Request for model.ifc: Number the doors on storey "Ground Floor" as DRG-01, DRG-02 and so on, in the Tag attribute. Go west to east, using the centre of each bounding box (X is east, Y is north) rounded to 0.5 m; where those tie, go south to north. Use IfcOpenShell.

First a look at what the model holds.

```python
import ifcopenshell
import ifcopenshell.util.element
import ifcopenshell.util.placement

model = ifcopenshell.open("model.ifc")
print(model.schema)
storey = next(s for s in model.by_type("IfcBuildingStorey") if s.Name == "Ground Floor")
doors = [e for e in ifcopenshell.util.element.get_decomposition(storey) if e.is_a("IfcDoor")]
for e in sorted(doors, key=lambda e: e.id()):
    origin = ifcopenshell.util.placement.get_local_placement(e.ObjectPlacement)[:3, 3]
    print(e.id(), e.Tag, e.Name, origin.round(2) + 0.0, sep=" | ")
```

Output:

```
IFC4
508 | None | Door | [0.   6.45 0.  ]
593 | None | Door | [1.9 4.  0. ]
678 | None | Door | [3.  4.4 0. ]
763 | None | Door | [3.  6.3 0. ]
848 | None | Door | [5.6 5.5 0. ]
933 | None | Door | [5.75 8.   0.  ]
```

```python
import ifcopenshell
import ifcopenshell.geom
import ifcopenshell.util.element
import ifcopenshell.util.shape

model = ifcopenshell.open("model.ifc")
settings = ifcopenshell.geom.settings()
settings.set("use-world-coords", True)


def centre(element):
    shape = ifcopenshell.geom.create_shape(settings, element)
    return ifcopenshell.util.shape.get_bbox_centroid(shape.geometry)


storey = next(s for s in model.by_type("IfcBuildingStorey") if s.Name == "Ground Floor")
doors = [e for e in ifcopenshell.util.element.get_decomposition(storey) if e.is_a("IfcDoor")]

# Insertion points can sit at a corner or the storey origin, so sort by the geometry (in metres).
centres = {e: centre(e) for e in doors}
doors.sort(key=lambda e: (round(centres[e][0] / 0.5), centres[e][1]))

for i, e in enumerate(doors, start=1):
    number = f"DRG-{i:02d}"
    e.Tag = number
    print(e.id(), number)

model.write("model_v2.ifc")
```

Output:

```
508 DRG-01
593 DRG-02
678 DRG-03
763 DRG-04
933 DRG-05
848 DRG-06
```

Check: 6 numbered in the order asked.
